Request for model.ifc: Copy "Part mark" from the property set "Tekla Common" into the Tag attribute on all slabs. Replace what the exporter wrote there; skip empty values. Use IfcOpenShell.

First a look at what the model holds.

```python
import ifcopenshell
import ifcopenshell.util.element

model = ifcopenshell.open("model.ifc")
print(model.schema)
slabs = model.by_type("IfcSlab")
print(len(slabs), "slabs")
for e in slabs[:8]:
    source = ifcopenshell.util.element.get_pset(e, "Tekla Common", "Part mark")
    target = e.Tag
    print(e.id(), repr(source), repr(target), sep=" | ")
```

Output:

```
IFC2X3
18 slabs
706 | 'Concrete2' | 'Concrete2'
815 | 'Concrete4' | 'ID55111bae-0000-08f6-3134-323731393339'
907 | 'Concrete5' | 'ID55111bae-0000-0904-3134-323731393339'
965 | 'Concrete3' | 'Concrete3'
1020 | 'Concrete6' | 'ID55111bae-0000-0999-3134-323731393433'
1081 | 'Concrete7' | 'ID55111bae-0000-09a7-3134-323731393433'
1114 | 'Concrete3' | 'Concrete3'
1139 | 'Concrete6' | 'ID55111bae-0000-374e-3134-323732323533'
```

```python
import ifcopenshell
import ifcopenshell.util.element

model = ifcopenshell.open("model.ifc")

count = 0
for e in model.by_type("IfcSlab"):
    value = ifcopenshell.util.element.get_pset(e, "Tekla Common", "Part mark")
    current = e.Tag
    if not value or not value.strip() or current == value:
        continue
    e.Tag = value
    count += 1

print(count, "slabs updated")

model.write("model_rev.ifc")
```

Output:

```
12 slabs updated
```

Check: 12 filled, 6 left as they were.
